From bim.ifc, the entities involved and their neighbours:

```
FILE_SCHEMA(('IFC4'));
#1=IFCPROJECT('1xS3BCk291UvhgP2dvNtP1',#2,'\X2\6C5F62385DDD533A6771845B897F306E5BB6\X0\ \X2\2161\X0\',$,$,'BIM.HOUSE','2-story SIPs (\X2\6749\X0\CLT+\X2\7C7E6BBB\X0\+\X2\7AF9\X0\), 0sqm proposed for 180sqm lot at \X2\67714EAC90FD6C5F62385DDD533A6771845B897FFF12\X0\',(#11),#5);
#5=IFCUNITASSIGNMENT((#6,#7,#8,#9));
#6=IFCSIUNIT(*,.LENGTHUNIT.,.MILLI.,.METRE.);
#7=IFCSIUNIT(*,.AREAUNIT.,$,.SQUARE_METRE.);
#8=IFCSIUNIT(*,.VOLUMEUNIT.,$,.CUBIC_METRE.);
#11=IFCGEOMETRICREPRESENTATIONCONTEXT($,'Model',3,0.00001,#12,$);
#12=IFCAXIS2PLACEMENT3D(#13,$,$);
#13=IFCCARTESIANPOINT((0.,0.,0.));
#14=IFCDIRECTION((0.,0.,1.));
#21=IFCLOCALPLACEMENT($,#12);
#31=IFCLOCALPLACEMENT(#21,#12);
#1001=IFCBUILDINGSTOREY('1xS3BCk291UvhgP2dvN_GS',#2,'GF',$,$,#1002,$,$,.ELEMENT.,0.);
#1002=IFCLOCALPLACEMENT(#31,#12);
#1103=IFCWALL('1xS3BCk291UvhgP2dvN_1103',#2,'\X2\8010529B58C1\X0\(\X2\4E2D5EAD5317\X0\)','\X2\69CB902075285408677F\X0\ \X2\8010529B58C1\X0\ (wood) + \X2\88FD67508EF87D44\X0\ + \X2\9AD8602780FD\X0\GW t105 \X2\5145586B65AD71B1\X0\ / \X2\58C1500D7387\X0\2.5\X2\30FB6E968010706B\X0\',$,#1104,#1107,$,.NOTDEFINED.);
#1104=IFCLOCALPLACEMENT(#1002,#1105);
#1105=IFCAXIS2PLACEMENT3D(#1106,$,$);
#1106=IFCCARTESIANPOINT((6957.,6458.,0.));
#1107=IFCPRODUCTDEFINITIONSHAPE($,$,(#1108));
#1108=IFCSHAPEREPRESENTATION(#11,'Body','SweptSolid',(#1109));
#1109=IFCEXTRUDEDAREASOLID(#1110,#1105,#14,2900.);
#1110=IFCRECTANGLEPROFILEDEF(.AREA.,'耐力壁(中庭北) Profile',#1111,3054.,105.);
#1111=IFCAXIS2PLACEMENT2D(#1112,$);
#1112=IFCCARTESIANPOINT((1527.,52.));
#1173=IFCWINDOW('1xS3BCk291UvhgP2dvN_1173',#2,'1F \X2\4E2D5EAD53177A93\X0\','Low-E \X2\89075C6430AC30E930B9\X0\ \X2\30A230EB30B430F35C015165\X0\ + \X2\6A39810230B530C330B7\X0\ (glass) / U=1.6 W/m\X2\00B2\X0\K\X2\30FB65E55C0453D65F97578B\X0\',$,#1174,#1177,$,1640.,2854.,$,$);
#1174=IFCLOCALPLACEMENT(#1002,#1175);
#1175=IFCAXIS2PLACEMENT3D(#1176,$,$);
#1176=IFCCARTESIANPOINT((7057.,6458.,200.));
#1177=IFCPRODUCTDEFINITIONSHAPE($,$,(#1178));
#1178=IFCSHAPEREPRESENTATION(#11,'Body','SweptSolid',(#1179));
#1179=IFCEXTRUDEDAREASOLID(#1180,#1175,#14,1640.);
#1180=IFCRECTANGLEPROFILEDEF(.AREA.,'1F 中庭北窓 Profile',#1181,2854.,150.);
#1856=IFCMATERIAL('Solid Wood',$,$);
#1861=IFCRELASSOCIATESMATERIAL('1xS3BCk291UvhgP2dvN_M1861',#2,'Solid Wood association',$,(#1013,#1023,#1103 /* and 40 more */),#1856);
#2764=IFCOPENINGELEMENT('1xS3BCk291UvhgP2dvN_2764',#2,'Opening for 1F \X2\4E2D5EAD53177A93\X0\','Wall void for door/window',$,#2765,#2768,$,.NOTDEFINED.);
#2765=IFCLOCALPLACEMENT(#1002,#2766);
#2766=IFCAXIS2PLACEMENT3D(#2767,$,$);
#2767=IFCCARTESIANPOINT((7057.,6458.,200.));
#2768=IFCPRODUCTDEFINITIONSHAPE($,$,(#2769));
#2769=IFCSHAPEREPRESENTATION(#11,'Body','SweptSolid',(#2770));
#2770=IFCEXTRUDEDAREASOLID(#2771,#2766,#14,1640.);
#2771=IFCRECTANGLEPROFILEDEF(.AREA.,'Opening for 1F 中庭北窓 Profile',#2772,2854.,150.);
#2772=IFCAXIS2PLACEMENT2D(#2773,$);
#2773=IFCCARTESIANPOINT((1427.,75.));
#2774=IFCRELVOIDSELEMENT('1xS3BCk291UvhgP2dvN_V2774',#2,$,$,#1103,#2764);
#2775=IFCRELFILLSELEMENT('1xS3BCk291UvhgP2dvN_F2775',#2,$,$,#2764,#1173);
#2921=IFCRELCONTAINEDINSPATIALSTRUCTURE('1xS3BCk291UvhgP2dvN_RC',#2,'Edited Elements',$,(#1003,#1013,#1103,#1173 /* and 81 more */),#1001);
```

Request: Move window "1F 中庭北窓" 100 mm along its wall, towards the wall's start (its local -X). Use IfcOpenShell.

```python
import ifcopenshell
import ifcopenshell.api.geometry
import ifcopenshell.util.placement
import ifcopenshell.util.unit

model = ifcopenshell.open("bim.ifc")
unit_scale = ifcopenshell.util.unit.calculate_unit_scale(model)

window = model.by_guid("1xS3BCk291UvhgP2dvN_1173")
opening = window.FillsVoids[0].RelatingOpeningElement
wall = opening.VoidsElements[0].RelatingBuildingElement

wall_matrix = ifcopenshell.util.placement.get_local_placement(wall.ObjectPlacement)
shift = wall_matrix[:3, 0] * -0.1 / unit_scale
before = ifcopenshell.util.placement.get_local_placement(window.ObjectPlacement)[:3, 3].copy()

# The window is not placed relative to its opening, so move both.
for product in (opening, window):
    matrix = ifcopenshell.util.placement.get_local_placement(product.ObjectPlacement)
    matrix[:3, 3] += shift
    ifcopenshell.api.geometry.edit_object_placement(model, product=product, matrix=matrix, is_si=False)

after = ifcopenshell.util.placement.get_local_placement(window.ObjectPlacement)[:3, 3]
print("window moved by", (after - before).round(3) + 0.0)

model.write("bim_v2.ifc")
```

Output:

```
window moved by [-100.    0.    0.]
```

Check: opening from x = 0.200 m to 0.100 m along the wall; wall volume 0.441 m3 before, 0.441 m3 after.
